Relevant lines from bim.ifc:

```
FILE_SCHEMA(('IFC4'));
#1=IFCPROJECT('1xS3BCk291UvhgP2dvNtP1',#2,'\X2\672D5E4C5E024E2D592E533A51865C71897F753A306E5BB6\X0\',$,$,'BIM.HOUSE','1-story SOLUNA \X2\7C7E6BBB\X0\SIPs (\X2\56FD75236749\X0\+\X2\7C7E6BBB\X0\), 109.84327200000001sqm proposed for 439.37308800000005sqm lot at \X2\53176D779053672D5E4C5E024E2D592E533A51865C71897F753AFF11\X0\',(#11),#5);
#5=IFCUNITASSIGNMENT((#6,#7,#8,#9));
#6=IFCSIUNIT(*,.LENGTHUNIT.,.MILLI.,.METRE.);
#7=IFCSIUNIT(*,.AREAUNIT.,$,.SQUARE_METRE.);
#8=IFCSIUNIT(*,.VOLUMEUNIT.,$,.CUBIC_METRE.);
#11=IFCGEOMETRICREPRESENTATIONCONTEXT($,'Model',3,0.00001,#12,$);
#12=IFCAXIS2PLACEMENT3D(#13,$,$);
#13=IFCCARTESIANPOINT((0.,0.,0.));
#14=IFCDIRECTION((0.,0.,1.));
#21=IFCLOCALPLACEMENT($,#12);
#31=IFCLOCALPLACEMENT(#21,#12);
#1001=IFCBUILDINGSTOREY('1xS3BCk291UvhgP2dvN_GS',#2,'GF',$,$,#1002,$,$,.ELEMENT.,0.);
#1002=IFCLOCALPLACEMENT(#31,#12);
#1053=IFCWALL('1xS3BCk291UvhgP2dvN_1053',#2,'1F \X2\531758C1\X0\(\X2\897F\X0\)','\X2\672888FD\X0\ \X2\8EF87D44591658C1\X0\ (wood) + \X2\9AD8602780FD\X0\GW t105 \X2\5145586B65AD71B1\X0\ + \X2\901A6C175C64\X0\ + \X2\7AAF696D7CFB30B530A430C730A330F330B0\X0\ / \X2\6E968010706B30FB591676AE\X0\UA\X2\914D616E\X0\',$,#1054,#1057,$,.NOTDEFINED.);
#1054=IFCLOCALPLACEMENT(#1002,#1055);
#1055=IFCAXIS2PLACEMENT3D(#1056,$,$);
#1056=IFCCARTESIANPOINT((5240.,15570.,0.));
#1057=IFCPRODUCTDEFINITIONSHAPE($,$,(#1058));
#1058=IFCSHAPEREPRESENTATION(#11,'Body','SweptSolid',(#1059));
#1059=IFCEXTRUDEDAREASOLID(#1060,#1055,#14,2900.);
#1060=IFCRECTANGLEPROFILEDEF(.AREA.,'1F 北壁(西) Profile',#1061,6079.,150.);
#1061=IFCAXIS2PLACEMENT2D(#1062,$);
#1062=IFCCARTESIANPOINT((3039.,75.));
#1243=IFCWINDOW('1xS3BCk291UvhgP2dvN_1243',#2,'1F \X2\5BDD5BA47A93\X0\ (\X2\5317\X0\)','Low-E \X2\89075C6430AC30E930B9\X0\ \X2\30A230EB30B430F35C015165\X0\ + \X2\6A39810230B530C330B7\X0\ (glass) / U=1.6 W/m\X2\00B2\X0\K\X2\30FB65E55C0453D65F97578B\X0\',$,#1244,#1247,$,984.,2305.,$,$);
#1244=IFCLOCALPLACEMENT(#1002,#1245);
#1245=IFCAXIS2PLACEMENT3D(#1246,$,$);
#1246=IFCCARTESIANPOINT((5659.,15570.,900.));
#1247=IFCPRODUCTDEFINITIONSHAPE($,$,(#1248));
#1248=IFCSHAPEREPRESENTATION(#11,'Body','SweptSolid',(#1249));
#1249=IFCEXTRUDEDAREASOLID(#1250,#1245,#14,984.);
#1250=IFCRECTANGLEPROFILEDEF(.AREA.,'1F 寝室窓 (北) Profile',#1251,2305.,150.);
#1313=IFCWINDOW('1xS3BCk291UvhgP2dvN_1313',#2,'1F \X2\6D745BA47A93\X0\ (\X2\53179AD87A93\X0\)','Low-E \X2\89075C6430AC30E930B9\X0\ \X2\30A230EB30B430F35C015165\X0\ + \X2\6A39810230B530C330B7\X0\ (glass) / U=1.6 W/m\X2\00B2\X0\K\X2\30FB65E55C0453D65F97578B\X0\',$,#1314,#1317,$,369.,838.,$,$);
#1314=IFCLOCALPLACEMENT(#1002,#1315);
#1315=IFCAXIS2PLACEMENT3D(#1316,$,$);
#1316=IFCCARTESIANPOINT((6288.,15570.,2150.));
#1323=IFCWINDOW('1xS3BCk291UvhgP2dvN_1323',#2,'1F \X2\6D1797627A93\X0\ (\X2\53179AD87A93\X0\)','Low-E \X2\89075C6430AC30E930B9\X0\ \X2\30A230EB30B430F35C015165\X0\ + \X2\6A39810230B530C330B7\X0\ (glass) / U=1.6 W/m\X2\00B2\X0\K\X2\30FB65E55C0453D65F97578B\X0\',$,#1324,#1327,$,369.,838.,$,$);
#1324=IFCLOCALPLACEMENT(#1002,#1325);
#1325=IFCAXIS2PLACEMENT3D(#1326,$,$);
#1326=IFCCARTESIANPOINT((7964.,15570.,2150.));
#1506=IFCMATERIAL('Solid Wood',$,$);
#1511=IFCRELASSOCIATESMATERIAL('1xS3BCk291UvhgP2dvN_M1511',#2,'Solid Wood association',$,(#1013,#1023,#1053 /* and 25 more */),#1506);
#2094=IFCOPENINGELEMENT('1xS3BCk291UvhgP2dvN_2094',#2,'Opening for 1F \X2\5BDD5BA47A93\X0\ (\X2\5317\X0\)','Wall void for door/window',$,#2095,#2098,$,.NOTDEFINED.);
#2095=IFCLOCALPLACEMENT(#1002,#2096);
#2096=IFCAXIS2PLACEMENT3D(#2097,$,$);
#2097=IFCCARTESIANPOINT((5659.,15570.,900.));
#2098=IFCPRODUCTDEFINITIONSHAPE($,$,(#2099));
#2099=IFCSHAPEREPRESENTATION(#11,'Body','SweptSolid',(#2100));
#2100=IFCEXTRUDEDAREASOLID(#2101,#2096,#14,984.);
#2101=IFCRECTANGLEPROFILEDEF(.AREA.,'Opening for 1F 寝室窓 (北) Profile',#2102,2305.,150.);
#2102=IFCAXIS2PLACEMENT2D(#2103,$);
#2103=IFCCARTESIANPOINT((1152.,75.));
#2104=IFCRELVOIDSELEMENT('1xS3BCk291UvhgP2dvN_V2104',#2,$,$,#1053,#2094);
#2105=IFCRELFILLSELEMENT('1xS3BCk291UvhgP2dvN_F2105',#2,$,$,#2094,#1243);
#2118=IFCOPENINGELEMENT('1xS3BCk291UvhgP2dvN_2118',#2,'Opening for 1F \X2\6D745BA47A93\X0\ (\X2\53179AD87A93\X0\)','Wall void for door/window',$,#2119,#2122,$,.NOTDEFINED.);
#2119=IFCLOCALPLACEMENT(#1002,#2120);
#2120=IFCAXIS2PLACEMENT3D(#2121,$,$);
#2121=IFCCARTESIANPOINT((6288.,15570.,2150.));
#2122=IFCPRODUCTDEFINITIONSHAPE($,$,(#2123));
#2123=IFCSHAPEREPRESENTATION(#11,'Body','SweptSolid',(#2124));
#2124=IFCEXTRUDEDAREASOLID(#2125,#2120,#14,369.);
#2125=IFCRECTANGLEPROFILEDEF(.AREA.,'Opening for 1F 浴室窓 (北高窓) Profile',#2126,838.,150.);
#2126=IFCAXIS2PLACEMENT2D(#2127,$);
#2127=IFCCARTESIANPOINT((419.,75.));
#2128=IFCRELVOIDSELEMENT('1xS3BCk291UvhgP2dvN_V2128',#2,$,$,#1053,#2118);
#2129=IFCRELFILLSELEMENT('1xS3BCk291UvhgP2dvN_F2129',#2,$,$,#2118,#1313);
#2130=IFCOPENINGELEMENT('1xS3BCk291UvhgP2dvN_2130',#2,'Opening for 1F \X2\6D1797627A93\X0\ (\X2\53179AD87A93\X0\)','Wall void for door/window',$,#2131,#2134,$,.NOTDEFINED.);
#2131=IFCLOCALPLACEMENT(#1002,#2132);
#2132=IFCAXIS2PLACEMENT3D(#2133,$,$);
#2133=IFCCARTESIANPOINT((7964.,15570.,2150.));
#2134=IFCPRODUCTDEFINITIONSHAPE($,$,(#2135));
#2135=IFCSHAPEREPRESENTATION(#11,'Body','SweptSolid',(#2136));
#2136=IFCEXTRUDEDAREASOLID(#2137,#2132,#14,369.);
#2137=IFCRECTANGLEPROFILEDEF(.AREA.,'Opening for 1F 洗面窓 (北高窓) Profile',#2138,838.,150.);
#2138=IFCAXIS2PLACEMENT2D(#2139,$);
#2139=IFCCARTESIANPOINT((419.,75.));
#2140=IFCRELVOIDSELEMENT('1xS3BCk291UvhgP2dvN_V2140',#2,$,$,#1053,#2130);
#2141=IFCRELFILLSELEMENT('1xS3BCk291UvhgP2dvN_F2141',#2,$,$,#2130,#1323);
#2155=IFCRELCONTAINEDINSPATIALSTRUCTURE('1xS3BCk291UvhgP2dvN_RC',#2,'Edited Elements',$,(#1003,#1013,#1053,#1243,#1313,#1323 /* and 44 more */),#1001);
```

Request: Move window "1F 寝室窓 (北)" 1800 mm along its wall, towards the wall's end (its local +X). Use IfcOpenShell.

```python
import ifcopenshell
import ifcopenshell.api.geometry
import ifcopenshell.util.placement

model = ifcopenshell.open("bim.ifc")

window = model.by_guid("1xS3BCk291UvhgP2dvN_1243")
opening = window.FillsVoids[0].RelatingOpeningElement
wall = opening.VoidsElements[0].RelatingBuildingElement

wall_matrix = ifcopenshell.util.placement.get_local_placement(wall.ObjectPlacement)
shift = wall_matrix[:3, 0] * 1800.0
before = ifcopenshell.util.placement.get_local_placement(window.ObjectPlacement)[:3, 3].copy()

# The window is not placed relative to its opening, so move both.
for product in (opening, window):
    matrix = ifcopenshell.util.placement.get_local_placement(product.ObjectPlacement)
    matrix[:3, 3] += shift
    ifcopenshell.api.geometry.edit_object_placement(model, product=product, matrix=matrix, is_si=False)

after = ifcopenshell.util.placement.get_local_placement(window.ObjectPlacement)[:3, 3]
print("window moved by", (after - before).round(3) + 0.0)

model.write("bim_updated.ifc")
```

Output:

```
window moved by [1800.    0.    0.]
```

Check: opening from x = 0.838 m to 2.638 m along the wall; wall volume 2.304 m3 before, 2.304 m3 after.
